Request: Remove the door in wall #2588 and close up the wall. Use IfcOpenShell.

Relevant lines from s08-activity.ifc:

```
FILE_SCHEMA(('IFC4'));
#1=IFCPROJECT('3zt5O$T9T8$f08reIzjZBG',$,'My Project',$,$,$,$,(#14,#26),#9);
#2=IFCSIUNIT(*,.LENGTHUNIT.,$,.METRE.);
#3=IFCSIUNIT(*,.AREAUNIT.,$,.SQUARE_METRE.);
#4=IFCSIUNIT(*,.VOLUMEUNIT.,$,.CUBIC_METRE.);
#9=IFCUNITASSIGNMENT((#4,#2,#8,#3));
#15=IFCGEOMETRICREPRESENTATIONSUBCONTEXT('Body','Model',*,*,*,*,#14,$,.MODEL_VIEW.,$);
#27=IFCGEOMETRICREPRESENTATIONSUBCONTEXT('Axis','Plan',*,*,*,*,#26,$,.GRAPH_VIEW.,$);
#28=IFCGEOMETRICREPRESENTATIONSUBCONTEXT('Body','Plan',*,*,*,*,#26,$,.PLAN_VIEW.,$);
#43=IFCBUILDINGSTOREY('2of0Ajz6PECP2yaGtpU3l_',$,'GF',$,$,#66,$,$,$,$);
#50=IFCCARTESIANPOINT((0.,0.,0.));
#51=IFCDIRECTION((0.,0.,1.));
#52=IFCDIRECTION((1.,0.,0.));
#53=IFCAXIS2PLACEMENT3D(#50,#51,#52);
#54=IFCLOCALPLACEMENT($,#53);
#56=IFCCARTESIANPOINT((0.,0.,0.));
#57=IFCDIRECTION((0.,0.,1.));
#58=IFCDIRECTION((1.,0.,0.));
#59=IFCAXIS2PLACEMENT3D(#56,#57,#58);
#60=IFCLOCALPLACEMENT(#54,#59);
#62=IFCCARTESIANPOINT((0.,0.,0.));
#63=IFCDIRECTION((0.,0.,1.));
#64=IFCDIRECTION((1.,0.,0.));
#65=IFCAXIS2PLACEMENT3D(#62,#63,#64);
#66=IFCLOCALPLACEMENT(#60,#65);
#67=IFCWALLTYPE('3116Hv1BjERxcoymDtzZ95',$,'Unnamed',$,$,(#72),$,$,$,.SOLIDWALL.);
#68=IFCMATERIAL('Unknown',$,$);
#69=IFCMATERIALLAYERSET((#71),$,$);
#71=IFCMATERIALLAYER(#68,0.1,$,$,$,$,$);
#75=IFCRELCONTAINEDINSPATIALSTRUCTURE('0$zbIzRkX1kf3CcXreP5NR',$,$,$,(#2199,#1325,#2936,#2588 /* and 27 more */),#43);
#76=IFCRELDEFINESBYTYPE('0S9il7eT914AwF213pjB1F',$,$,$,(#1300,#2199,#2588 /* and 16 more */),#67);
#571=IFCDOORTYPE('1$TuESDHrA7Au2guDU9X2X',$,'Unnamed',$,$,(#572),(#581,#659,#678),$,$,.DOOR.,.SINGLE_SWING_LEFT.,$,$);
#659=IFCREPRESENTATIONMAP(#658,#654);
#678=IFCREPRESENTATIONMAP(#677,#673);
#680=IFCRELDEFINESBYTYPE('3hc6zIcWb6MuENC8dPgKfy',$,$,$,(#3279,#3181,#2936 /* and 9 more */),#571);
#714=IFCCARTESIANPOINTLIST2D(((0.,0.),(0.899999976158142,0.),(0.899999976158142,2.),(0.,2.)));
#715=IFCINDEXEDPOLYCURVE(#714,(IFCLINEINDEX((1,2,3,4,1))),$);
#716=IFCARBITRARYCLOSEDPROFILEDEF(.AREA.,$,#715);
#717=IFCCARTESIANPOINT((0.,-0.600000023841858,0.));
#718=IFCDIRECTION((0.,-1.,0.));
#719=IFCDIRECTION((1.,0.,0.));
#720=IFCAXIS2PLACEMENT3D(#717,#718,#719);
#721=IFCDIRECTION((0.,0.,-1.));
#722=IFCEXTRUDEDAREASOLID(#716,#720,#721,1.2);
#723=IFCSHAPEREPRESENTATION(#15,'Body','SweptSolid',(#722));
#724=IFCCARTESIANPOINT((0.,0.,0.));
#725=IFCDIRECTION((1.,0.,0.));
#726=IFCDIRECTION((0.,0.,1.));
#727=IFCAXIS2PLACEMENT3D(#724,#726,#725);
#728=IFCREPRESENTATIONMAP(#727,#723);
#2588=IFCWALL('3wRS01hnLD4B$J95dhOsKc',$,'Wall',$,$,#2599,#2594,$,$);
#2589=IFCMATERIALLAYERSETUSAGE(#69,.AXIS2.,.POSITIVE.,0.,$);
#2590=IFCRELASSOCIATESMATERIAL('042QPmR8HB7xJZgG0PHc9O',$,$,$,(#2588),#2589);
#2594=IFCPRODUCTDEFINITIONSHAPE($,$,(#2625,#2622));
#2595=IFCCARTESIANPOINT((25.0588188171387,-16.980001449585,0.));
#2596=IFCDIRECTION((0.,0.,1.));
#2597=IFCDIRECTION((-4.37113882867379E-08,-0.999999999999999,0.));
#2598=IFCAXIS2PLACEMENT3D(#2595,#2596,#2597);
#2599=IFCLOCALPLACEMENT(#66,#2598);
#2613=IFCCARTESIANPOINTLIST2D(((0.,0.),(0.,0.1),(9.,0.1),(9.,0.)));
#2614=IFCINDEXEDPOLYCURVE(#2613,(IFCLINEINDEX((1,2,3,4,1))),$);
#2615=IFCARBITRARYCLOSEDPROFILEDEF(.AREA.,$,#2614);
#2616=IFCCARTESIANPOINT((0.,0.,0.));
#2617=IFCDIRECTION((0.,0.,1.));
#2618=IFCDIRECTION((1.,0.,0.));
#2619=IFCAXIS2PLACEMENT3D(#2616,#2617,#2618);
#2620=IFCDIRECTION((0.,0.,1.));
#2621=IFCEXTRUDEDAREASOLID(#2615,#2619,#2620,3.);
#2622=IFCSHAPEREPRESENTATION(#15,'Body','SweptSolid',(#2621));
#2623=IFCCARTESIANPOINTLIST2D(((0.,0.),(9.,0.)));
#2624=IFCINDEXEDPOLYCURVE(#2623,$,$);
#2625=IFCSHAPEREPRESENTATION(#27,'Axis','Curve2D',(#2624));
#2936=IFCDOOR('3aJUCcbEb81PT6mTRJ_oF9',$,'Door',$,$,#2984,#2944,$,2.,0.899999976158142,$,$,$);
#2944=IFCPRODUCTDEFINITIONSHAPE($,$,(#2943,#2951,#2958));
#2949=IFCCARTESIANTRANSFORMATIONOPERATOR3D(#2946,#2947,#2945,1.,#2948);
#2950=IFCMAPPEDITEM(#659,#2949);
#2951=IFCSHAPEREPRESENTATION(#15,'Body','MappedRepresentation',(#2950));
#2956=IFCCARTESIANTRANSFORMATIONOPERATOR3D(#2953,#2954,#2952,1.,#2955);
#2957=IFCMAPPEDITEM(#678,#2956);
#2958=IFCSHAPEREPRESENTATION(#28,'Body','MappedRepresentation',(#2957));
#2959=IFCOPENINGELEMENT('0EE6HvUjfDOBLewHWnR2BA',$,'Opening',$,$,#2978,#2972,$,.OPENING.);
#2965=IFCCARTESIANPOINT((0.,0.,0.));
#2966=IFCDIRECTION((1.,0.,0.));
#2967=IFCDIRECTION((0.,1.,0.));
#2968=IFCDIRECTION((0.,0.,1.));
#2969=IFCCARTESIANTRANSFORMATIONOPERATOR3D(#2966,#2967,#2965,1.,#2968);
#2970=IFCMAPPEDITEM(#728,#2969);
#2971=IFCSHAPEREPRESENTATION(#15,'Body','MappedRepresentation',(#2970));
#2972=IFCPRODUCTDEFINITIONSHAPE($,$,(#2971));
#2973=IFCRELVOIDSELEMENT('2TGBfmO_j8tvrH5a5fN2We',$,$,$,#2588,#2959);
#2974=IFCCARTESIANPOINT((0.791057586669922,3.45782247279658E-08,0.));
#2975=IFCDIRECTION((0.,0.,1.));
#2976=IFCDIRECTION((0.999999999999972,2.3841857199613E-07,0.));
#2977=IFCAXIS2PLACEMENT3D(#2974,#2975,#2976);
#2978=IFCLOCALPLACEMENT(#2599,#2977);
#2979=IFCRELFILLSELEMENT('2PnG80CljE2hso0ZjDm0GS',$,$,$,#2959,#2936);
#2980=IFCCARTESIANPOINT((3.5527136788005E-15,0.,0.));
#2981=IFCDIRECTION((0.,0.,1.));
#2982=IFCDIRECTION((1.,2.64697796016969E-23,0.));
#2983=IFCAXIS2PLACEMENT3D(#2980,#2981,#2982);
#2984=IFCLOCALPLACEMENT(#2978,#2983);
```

```python
import ifcopenshell
import ifcopenshell.api.feature
import ifcopenshell.api.root
import ifcopenshell.geom
import ifcopenshell.util.shape

model = ifcopenshell.open("s08-activity.ifc")
settings = ifcopenshell.geom.settings()


def volume(element):
    """Net volume in cubic metres, openings subtracted."""
    shape = ifcopenshell.geom.create_shape(settings, element)
    return ifcopenshell.util.shape.get_volume(shape.geometry)


door = model.by_guid("3aJUCcbEb81PT6mTRJ_oF9")
opening = door.FillsVoids[0].RelatingOpeningElement
wall = opening.VoidsElements[0].RelatingBuildingElement
before = volume(wall)

ifcopenshell.api.root.remove_product(model, product=door)
ifcopenshell.api.feature.remove_feature(model, feature=opening)

after = volume(wall)

print(f"wall volume {before:.3f} -> {after:.3f} m3")

model.write("s08-activity_updated.ifc")
```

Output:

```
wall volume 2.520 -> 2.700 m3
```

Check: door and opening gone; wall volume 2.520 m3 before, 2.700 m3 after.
